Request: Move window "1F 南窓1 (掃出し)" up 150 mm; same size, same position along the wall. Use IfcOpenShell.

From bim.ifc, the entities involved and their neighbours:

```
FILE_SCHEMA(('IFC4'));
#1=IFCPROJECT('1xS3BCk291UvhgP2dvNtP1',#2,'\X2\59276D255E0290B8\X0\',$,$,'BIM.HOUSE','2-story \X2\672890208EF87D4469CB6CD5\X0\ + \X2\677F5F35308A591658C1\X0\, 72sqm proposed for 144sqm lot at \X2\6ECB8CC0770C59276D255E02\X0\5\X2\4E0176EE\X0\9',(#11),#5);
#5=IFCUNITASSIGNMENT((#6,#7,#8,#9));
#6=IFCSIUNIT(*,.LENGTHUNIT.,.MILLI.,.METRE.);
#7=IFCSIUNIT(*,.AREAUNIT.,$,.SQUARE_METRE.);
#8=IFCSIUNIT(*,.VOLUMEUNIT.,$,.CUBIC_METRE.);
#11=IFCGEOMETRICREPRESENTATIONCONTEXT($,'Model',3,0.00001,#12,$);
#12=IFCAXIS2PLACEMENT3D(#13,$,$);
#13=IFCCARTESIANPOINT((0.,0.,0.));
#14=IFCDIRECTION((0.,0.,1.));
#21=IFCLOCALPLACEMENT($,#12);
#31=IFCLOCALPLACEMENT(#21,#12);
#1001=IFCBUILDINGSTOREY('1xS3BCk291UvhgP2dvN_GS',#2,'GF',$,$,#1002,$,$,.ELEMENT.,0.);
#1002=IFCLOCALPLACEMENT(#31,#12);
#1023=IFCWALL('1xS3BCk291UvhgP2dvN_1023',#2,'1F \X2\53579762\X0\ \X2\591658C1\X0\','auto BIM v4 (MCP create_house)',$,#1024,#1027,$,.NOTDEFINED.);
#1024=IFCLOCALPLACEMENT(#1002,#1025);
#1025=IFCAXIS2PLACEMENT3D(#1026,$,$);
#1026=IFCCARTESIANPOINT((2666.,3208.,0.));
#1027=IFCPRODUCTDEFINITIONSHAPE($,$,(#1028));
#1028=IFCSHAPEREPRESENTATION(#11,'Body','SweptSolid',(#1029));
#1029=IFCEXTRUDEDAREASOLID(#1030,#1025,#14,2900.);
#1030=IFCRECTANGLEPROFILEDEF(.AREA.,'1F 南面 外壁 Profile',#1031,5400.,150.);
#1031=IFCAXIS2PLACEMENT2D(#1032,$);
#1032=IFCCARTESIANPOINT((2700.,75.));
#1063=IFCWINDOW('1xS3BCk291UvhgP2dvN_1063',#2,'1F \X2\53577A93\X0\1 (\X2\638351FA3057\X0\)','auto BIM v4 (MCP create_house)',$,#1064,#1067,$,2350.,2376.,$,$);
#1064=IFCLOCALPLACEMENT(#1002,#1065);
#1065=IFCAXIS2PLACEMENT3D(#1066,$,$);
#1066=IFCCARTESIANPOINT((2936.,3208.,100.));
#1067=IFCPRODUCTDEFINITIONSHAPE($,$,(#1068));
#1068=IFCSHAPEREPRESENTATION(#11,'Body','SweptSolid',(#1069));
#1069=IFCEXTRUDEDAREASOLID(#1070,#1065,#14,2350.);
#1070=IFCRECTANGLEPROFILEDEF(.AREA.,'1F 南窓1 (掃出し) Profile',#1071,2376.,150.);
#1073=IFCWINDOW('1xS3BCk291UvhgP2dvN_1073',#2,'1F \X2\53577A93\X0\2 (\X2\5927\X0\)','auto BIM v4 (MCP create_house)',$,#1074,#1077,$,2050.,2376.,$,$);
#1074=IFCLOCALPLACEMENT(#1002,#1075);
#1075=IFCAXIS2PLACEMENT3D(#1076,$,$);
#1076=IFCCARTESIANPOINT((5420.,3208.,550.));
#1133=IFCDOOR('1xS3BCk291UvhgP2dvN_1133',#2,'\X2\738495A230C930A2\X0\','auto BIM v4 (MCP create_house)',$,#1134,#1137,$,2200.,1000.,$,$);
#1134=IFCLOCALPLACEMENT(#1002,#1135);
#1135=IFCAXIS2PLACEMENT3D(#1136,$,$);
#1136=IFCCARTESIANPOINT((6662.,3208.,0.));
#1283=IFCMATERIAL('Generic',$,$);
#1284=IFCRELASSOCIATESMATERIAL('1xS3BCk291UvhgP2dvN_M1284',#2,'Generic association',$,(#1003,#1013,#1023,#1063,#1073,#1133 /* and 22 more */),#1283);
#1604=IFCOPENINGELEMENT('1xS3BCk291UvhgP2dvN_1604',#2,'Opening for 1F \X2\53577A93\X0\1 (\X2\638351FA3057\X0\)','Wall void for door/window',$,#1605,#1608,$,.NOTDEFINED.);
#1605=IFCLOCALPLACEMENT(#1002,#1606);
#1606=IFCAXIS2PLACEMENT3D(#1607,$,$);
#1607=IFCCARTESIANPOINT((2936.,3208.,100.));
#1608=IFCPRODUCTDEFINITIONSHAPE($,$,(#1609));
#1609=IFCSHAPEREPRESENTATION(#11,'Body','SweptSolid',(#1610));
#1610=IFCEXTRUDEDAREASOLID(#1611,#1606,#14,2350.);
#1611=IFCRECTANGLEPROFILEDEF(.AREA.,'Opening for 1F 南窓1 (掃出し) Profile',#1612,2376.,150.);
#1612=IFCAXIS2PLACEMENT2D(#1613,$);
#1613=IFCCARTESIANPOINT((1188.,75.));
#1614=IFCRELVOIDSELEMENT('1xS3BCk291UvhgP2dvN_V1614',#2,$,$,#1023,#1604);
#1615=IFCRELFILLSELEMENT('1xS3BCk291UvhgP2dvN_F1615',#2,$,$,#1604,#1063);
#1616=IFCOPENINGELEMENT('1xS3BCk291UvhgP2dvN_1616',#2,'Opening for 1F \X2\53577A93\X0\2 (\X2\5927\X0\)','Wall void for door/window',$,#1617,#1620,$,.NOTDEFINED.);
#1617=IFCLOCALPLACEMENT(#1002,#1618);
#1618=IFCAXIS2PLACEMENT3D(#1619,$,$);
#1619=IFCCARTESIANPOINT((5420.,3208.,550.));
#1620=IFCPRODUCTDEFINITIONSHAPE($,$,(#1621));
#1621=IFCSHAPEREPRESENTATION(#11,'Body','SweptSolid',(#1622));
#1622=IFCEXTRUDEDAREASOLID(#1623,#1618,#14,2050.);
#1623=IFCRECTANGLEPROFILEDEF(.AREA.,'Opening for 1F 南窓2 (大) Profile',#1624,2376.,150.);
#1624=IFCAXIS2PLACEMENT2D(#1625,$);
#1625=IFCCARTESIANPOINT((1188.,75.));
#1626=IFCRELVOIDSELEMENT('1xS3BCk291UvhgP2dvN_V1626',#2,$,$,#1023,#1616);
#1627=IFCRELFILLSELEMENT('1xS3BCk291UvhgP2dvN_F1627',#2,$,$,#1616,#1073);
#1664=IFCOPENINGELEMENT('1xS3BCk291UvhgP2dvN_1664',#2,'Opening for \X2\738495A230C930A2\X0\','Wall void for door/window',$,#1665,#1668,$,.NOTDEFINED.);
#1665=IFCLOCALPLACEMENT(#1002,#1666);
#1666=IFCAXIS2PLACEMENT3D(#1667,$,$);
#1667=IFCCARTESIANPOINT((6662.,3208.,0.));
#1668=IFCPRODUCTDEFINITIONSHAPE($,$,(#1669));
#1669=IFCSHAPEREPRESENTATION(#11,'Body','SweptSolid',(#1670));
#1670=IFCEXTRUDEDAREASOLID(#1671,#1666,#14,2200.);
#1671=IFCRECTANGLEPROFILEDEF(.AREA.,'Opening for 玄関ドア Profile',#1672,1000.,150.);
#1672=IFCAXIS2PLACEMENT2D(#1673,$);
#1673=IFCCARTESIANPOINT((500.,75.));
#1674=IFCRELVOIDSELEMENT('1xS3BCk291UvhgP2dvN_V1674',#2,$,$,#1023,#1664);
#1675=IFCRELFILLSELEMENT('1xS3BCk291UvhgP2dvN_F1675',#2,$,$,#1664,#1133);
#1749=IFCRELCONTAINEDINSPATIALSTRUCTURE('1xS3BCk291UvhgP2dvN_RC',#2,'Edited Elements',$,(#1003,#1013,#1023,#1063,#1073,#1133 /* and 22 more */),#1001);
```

```python
import numpy as np
import ifcopenshell
import ifcopenshell.api.geometry
import ifcopenshell.util.placement
import ifcopenshell.util.unit

model = ifcopenshell.open("bim.ifc")
unit_scale = ifcopenshell.util.unit.calculate_unit_scale(model)

window = model.by_guid("1xS3BCk291UvhgP2dvN_1063")
opening = window.FillsVoids[0].RelatingOpeningElement
dz = 0.15 / unit_scale

shift = np.array([0.0, 0.0, dz])
# The window is not placed relative to its opening, so move both.
for product in (opening, window):
    matrix = ifcopenshell.util.placement.get_local_placement(product.ObjectPlacement)
    matrix[:3, 3] += shift
    ifcopenshell.api.geometry.edit_object_placement(model, product=product, matrix=matrix, is_si=False)

print(f"moved by {dz * unit_scale:+.3f} m")

model.write("bim-out.ifc")
```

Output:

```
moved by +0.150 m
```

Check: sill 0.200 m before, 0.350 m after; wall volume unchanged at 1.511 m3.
